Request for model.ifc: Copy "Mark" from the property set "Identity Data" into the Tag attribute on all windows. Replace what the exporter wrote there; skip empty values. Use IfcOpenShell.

First a look at what the model holds.

```python
import ifcopenshell
import ifcopenshell.util.element

model = ifcopenshell.open("model.ifc")
print(model.schema)
windows = model.by_type("IfcWindow")
print(len(windows), "windows")
for e in windows[:8]:
    source = ifcopenshell.util.element.get_pset(e, "Identity Data", "Mark")
    target = e.Tag
    print(e.id(), repr(source), repr(target), sep=" | ")
```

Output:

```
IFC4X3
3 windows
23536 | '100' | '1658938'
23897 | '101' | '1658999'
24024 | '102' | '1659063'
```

```python
import ifcopenshell
import ifcopenshell.util.element

model = ifcopenshell.open("model.ifc")

count = 0
for e in model.by_type("IfcWindow"):
    value = ifcopenshell.util.element.get_pset(e, "Identity Data", "Mark")
    current = e.Tag
    if not value or not value.strip() or current == value:
        continue
    e.Tag = value
    count += 1

print(count, "windows updated")

model.write("model_v2.ifc")
```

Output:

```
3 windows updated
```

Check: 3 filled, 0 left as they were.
